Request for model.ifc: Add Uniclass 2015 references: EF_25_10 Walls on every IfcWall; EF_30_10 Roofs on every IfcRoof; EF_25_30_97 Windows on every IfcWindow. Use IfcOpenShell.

First a look at what the model holds.

```python
import ifcopenshell

model = ifcopenshell.open("model.ifc")
print(model.schema)
print("classifications:", [c.Name for c in model.by_type("IfcClassification")])
for ifc_class in ("IfcDoor", "IfcRoof", "IfcStair", "IfcWall", "IfcWindow"):
    print(ifc_class, len(model.by_type(ifc_class)))
```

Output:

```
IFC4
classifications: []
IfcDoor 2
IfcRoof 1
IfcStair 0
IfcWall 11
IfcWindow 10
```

```python
import ifcopenshell
import ifcopenshell.api.classification

model = ifcopenshell.open("model.ifc")

system = ifcopenshell.api.classification.add_classification(model, classification="Uniclass 2015")

codes = {
    "IfcWall": ("EF_25_10", "Walls"),
    "IfcRoof": ("EF_30_10", "Roofs"),
    "IfcWindow": ("EF_25_30_97", "Windows"),
}
for ifc_class, (code, name) in codes.items():
    products = model.by_type(ifc_class)
    ifcopenshell.api.classification.add_reference(
        model, products=products, classification=system, identification=code, name=name
    )
    print(code, len(products))

model.write("model_v2.ifc")
```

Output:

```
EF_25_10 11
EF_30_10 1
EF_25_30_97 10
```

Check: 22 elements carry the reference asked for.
